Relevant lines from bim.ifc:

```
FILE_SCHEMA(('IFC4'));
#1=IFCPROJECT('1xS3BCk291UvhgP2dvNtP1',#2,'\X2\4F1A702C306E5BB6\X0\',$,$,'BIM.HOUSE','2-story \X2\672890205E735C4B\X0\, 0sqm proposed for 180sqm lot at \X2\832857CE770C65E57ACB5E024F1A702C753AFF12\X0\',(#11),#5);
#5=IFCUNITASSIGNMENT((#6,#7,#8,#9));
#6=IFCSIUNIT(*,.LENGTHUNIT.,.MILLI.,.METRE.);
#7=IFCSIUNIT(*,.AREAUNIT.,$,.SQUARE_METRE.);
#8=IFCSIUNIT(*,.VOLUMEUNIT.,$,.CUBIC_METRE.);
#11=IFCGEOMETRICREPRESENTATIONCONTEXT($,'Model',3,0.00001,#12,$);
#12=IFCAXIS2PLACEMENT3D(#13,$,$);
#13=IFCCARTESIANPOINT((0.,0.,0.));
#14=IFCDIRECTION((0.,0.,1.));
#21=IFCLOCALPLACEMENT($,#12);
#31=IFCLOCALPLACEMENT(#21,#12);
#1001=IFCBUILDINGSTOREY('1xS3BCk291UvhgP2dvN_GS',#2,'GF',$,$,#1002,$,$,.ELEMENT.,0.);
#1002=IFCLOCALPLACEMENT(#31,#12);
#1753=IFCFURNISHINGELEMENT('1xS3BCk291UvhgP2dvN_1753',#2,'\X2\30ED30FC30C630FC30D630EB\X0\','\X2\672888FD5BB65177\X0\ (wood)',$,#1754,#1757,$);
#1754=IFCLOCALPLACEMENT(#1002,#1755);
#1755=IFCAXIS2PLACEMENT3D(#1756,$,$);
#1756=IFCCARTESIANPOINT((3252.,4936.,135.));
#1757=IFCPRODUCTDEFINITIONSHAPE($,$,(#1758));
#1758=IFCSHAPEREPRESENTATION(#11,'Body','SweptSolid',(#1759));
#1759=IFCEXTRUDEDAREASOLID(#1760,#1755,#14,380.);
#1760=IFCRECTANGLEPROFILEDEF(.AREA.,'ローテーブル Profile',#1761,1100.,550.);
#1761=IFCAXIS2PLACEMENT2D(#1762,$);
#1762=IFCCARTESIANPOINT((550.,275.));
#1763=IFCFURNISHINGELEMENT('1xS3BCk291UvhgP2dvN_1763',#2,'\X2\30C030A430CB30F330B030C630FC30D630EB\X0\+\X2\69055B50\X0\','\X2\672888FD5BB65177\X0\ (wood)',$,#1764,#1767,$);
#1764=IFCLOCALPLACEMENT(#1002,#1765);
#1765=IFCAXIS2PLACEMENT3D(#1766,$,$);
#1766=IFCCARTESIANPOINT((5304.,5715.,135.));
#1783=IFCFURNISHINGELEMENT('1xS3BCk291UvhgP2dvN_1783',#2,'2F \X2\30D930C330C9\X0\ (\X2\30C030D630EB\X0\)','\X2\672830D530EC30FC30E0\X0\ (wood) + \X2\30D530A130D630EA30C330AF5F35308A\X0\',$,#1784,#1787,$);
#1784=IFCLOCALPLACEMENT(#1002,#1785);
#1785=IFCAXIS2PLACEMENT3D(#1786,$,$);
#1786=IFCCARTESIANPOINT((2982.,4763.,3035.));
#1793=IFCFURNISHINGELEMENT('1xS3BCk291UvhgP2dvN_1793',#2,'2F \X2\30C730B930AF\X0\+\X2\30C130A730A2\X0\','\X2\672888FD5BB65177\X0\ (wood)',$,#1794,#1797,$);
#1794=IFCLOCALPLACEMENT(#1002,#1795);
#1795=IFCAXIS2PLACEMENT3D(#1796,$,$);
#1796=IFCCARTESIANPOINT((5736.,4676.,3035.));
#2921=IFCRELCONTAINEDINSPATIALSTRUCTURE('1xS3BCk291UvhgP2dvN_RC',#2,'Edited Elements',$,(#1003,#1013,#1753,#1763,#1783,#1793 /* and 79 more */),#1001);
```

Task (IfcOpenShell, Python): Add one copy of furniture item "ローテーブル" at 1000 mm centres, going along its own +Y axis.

```python
import ifcopenshell
import ifcopenshell.api.geometry
import ifcopenshell.api.root
import ifcopenshell.util.element
import ifcopenshell.util.placement
import ifcopenshell.util.unit

model = ifcopenshell.open("bim.ifc")
unit_scale = ifcopenshell.util.unit.calculate_unit_scale(model)


def reuse_history(source, copy):
    """copy_class also copies each property set's owner history, people and application; keep the originals."""
    for rel in copy.IsDefinedBy:
        if rel.is_a("IfcRelDefinesByProperties") and (history := rel.RelatingPropertyDefinition.OwnerHistory):
            rel.RelatingPropertyDefinition.OwnerHistory = source.OwnerHistory
            ifcopenshell.util.element.remove_deep2(model, history)


source = model.by_guid("1xS3BCk291UvhgP2dvN_1753")
base = ifcopenshell.util.placement.get_local_placement(source.ObjectPlacement)
step = base[:3, 1] * 1 / unit_scale

for i in range(1, 2):
    copy = ifcopenshell.api.root.copy_class(model, product=source)
    copy.Representation = ifcopenshell.util.element.copy_deep(
        model, source.Representation, exclude=["IfcGeometricRepresentationContext", "IfcRepresentationMap"]
    )
    reuse_history(source, copy)
    matrix = base.copy()
    matrix[:3, 3] += i * step
    print("added at", matrix[:3, 3].round(3) + 0.0)
    ifcopenshell.api.geometry.edit_object_placement(model, product=copy, matrix=matrix, is_si=False)

model.write("bim_rev.ifc")
```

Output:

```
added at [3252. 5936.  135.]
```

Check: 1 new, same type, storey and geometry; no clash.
